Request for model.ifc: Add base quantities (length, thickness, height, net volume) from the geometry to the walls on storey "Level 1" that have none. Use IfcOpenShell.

First a look at what the model holds.

```python
import ifcopenshell
import ifcopenshell.util.element
import ifcopenshell.util.unit

model = ifcopenshell.open("model.ifc")
print(model.schema)
for unit_type in ("LENGTHUNIT", "AREAUNIT", "VOLUMEUNIT"):
    print(unit_type, ifcopenshell.util.unit.calculate_unit_scale(model, unit_type))
storey = next(s for s in model.by_type("IfcBuildingStorey") if s.Name == "Level 1")
walls = [e for e in ifcopenshell.util.element.get_decomposition(storey) if e.is_a("IfcWall")]
for e in sorted(walls, key=lambda e: e.id()):
    print(e.id(), e.is_a(), e.Name, list(ifcopenshell.util.element.get_psets(e, qtos_only=True)), sep=" | ")
```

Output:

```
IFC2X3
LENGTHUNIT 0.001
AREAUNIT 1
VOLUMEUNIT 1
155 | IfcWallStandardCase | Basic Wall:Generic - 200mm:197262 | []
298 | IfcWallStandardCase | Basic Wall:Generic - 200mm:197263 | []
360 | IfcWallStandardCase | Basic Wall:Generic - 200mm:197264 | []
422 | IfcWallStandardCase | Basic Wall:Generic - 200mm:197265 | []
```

```python
import ifcopenshell
import ifcopenshell.api.pset
import ifcopenshell.geom
import ifcopenshell.util.element
import ifcopenshell.util.shape
import ifcopenshell.util.unit

model = ifcopenshell.open("model.ifc")
unit_scale = ifcopenshell.util.unit.calculate_unit_scale(model)
volume_scale = ifcopenshell.util.unit.calculate_unit_scale(model, "VOLUMEUNIT")
settings = ifcopenshell.geom.settings()

storey = next(s for s in model.by_type("IfcBuildingStorey") if s.Name == "Level 1")
walls = [e for e in ifcopenshell.util.element.get_decomposition(storey) if e.is_a("IfcWall")]

for e in sorted(walls, key=lambda e: e.id()):
    if ifcopenshell.util.element.get_psets(e, qtos_only=True, should_inherit=False):
        continue
    # Geometry comes back in metres, in the element's own axes.
    shape = ifcopenshell.geom.create_shape(settings, e)
    values = {
        "Length": ifcopenshell.util.shape.get_x(shape.geometry) / unit_scale,
        "Width": ifcopenshell.util.shape.get_y(shape.geometry) / unit_scale,
        "Height": ifcopenshell.util.shape.get_z(shape.geometry) / unit_scale,
        "NetVolume": ifcopenshell.util.shape.get_volume(shape.geometry) / volume_scale,
    }
    qto = ifcopenshell.api.pset.add_qto(model, product=e, name="BaseQuantities")
    ifcopenshell.api.pset.edit_qto(model, qto=qto, properties=values)
    print(e.id(), {k: round(v, 3) for k, v in values.items()})

model.write("model_v2.ifc")
```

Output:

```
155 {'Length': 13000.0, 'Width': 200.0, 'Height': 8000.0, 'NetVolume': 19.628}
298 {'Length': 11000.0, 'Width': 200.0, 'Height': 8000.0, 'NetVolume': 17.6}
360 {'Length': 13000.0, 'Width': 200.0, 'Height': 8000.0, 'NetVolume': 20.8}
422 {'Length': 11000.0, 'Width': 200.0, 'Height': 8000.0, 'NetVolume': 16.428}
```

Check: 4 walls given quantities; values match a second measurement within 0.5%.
